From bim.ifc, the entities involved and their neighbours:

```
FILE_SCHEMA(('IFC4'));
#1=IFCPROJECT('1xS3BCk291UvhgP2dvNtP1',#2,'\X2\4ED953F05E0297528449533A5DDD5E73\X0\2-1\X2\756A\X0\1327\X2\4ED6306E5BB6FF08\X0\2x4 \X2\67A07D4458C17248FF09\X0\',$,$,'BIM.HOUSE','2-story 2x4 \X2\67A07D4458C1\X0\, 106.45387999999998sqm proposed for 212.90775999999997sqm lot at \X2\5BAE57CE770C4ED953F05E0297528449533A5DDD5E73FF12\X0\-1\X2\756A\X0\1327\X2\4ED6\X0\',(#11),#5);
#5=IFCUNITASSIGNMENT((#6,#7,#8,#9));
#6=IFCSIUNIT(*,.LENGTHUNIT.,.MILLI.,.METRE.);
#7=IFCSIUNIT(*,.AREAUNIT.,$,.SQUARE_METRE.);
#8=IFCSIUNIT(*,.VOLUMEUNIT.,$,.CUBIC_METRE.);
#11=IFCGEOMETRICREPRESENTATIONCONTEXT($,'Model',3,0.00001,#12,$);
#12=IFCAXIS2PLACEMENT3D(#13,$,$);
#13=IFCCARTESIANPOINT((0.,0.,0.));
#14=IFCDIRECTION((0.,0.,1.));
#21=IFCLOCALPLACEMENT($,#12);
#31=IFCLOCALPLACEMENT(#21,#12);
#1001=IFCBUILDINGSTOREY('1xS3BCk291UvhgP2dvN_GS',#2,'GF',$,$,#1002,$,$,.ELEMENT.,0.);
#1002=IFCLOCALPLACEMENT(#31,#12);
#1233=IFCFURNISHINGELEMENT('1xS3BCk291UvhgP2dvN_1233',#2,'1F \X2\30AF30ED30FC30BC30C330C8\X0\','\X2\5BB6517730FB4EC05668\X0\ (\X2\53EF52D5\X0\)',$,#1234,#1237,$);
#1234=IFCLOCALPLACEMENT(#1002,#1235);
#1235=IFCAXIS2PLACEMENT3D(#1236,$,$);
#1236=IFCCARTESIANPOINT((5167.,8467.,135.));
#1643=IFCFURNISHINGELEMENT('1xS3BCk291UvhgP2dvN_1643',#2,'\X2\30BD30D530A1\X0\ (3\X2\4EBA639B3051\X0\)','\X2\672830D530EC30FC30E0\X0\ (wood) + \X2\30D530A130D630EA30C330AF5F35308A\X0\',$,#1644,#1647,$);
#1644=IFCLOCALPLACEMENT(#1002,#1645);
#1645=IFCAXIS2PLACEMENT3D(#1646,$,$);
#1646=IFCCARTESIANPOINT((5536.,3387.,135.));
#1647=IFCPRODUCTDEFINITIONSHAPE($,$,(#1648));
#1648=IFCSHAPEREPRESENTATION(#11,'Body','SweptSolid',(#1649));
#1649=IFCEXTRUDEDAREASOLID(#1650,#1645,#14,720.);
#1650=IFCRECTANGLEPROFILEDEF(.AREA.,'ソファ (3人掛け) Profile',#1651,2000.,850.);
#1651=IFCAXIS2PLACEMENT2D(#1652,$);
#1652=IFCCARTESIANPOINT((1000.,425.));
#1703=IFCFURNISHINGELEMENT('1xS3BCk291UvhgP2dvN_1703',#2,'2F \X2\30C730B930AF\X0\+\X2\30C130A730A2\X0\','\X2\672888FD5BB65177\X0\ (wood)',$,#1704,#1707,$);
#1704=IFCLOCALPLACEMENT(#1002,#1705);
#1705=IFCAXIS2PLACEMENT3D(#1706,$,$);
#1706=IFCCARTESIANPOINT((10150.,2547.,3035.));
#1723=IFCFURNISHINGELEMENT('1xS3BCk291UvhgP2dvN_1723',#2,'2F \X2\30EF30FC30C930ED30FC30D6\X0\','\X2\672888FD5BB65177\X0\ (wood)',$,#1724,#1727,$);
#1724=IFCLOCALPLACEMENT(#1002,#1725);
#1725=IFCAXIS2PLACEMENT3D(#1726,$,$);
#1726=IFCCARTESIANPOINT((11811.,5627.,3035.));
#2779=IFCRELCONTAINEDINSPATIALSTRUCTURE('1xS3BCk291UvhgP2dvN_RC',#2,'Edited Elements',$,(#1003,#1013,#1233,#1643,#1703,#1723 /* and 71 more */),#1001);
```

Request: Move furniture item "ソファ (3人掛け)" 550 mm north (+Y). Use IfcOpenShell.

```python
import ifcopenshell
import ifcopenshell.api.geometry
import ifcopenshell.util.placement
import ifcopenshell.util.unit

model = ifcopenshell.open("bim.ifc")
unit_scale = ifcopenshell.util.unit.calculate_unit_scale(model)

item = model.by_id(1643)
matrix = ifcopenshell.util.placement.get_local_placement(item.ObjectPlacement)
matrix[1, 3] += 0.55 / unit_scale
ifcopenshell.api.geometry.edit_object_placement(model, product=item, matrix=matrix, is_si=False)

print(ifcopenshell.util.placement.get_local_placement(item.ObjectPlacement).round(3) + 0.0)

model.write("bim_edited.ifc")
```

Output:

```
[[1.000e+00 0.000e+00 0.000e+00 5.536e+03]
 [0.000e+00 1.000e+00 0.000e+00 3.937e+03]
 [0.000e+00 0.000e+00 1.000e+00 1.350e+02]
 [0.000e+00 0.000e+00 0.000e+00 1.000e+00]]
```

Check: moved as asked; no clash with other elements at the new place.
